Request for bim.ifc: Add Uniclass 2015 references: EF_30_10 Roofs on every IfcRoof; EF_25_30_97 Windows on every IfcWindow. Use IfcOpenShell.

First a look at what the model holds.

```python
import ifcopenshell

model = ifcopenshell.open("bim.ifc")
print(model.schema)
print("classifications:", [c.Name for c in model.by_type("IfcClassification")])
for ifc_class in ("IfcDoor", "IfcRoof", "IfcStair", "IfcWall", "IfcWindow"):
    print(ifc_class, len(model.by_type(ifc_class)))
```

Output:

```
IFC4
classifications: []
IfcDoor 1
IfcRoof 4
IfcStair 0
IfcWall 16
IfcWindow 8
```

```python
import ifcopenshell
import ifcopenshell.api.classification

model = ifcopenshell.open("bim.ifc")

system = ifcopenshell.api.classification.add_classification(model, classification="Uniclass 2015")

codes = {
    "IfcRoof": ("EF_30_10", "Roofs"),
    "IfcWindow": ("EF_25_30_97", "Windows"),
}
for ifc_class, (code, name) in codes.items():
    products = model.by_type(ifc_class)
    ifcopenshell.api.classification.add_reference(
        model, products=products, classification=system, identification=code, name=name
    )
    print(code, len(products))

model.write("bim_updated.ifc")
```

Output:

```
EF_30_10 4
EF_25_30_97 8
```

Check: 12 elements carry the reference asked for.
